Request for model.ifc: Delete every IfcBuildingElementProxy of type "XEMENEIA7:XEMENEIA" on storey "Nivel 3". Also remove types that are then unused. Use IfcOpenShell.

First a look at what the model holds.

```python
import ifcopenshell
import ifcopenshell.util.element

model = ifcopenshell.open("model.ifc")
print(model.schema)
storey = next(s for s in model.by_type("IfcBuildingStorey") if s.Name == "Nivel 3")
proxies = [e for e in ifcopenshell.util.element.get_decomposition(storey) if e.is_a("IfcBuildingElementProxy")]
seen = {}
for e in proxies:
    element_type = ifcopenshell.util.element.get_type(e)
    name = element_type.Name if element_type not in (None, e) else None
    seen[name] = seen.get(name, 0) + 1
for name, count in sorted(seen.items(), key=str):
    print(count, "x", name)
```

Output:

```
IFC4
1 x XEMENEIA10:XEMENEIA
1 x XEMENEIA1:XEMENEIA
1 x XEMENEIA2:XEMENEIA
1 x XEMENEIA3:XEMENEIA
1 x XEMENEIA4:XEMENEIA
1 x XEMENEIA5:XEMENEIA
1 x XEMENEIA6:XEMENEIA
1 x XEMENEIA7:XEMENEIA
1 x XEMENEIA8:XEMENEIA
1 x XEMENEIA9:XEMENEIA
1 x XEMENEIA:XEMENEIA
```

```python
import ifcopenshell
import ifcopenshell.api.root
import ifcopenshell.util.element

model = ifcopenshell.open("model.ifc")

storey = next(s for s in model.by_type("IfcBuildingStorey") if s.Name == "Nivel 3")
proxies = [e for e in ifcopenshell.util.element.get_decomposition(storey) if e.is_a("IfcBuildingElementProxy")]
targets = [e for e in proxies if (t := ifcopenshell.util.element.get_type(e)) not in (None, e) and t.Name == "XEMENEIA7:XEMENEIA"]
types = {ifcopenshell.util.element.get_type(e) for e in targets} - {None, *targets}

for e in targets:
    ifcopenshell.api.root.remove_product(model, product=e)
print(len(targets), "removed")

unused = [t for t in types if not ifcopenshell.util.element.get_types(t)]
for t in unused:
    ifcopenshell.api.root.remove_product(model, product=t)
print(len(unused), "unused types removed")

model.write("model-out.ifc")
```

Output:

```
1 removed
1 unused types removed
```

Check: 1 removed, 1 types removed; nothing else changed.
